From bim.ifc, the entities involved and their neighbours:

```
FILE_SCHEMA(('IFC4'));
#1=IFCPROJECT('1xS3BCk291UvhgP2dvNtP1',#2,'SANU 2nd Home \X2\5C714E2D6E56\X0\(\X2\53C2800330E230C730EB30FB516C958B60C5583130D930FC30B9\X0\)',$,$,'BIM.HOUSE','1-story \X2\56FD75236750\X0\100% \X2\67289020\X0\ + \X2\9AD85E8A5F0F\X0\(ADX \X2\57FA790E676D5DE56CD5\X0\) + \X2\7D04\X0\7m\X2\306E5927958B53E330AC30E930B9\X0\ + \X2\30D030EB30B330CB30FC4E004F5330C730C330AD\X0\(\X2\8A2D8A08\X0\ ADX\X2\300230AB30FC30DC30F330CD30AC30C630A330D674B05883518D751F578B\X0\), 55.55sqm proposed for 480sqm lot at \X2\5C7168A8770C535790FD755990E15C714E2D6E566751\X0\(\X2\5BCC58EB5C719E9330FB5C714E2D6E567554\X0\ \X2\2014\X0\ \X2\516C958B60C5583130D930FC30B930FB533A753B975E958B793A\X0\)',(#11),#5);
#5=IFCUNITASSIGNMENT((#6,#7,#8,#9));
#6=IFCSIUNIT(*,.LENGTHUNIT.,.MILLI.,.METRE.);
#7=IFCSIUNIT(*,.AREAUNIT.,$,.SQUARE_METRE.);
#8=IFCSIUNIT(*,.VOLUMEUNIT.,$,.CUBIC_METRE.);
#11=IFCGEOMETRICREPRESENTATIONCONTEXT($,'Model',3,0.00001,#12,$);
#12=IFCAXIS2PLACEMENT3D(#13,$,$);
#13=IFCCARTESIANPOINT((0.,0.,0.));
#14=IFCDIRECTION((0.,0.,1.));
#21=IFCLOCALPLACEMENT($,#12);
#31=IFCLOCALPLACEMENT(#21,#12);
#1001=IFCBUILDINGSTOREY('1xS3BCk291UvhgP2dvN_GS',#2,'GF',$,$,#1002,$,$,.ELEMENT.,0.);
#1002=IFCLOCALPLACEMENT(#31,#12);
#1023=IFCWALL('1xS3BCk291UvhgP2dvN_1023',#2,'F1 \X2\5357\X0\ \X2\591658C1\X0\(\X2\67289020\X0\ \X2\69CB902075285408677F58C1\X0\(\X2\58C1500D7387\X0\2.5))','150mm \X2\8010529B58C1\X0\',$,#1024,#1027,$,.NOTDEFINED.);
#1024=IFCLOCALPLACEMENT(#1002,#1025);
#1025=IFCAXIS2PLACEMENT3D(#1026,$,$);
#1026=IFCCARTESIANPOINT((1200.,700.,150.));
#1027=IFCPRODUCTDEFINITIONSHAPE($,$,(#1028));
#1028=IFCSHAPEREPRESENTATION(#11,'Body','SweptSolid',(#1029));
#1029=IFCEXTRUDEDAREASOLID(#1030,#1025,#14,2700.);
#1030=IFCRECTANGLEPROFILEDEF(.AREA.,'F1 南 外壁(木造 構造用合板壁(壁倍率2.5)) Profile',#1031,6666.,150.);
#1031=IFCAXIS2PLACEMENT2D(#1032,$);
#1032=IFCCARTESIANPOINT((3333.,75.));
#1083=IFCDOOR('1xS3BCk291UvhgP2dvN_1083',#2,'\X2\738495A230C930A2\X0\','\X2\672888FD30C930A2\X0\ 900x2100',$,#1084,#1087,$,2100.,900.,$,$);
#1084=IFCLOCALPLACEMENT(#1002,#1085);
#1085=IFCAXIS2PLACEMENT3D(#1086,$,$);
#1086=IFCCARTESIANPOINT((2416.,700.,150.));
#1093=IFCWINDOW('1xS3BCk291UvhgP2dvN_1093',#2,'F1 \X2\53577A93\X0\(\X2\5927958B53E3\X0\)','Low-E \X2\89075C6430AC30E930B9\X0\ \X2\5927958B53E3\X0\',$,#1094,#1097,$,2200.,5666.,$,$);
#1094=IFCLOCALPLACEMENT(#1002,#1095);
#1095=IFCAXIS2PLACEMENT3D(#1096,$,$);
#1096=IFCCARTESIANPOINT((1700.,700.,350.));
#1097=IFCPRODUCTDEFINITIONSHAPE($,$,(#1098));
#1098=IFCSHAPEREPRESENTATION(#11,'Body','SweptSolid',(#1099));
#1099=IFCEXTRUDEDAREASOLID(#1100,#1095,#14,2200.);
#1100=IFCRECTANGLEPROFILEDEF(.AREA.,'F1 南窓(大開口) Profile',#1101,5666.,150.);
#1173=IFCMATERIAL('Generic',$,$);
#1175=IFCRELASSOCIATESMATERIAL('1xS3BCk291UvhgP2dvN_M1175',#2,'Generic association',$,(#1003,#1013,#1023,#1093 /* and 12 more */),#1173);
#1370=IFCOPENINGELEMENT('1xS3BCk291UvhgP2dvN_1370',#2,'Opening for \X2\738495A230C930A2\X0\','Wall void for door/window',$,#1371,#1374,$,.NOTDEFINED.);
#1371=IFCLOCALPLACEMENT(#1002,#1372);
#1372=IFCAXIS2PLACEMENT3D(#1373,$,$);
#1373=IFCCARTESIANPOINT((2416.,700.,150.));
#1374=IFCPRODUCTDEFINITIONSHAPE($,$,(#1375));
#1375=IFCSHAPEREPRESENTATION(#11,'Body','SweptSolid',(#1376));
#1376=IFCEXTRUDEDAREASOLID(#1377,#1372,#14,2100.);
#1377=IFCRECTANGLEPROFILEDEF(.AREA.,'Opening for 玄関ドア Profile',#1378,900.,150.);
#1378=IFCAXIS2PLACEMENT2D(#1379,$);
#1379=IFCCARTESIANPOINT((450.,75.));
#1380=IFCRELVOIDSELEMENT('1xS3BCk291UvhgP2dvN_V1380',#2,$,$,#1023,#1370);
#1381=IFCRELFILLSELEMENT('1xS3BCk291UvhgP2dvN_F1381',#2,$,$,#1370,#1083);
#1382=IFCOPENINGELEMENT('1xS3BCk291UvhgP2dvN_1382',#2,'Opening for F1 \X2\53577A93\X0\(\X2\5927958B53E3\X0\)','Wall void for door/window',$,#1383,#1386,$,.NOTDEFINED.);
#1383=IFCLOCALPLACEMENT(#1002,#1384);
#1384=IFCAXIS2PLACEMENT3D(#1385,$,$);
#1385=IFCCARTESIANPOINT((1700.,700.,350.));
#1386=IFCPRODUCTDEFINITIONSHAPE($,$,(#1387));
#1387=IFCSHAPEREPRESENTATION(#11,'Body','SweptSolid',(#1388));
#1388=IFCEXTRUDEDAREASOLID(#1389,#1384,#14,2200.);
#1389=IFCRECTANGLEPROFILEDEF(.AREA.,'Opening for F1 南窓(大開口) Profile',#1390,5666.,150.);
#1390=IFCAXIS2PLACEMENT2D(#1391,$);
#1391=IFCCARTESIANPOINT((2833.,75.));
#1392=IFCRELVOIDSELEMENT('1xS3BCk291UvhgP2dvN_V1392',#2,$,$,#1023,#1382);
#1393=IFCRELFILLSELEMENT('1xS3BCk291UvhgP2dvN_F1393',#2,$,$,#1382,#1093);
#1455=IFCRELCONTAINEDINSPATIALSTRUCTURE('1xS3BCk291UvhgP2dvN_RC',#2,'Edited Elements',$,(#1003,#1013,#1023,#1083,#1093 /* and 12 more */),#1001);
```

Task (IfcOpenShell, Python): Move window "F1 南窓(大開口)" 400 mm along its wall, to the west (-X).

```python
import ifcopenshell
import ifcopenshell.api.geometry
import ifcopenshell.util.placement
import ifcopenshell.util.unit

model = ifcopenshell.open("bim.ifc")
unit_scale = ifcopenshell.util.unit.calculate_unit_scale(model)

window = model.by_guid("1xS3BCk291UvhgP2dvN_1093")
opening = window.FillsVoids[0].RelatingOpeningElement
wall = opening.VoidsElements[0].RelatingBuildingElement

wall_matrix = ifcopenshell.util.placement.get_local_placement(wall.ObjectPlacement)
shift = wall_matrix[:3, 0] * -0.4 / unit_scale
before = ifcopenshell.util.placement.get_local_placement(window.ObjectPlacement)[:3, 3].copy()

# The window is not placed relative to its opening, so move both.
for product in (opening, window):
    matrix = ifcopenshell.util.placement.get_local_placement(product.ObjectPlacement)
    matrix[:3, 3] += shift
    ifcopenshell.api.geometry.edit_object_placement(model, product=product, matrix=matrix, is_si=False)

after = ifcopenshell.util.placement.get_local_placement(window.ObjectPlacement)[:3, 3]
print("window moved by", (after - before).round(3) + 0.0)

model.write("bim_rev.ifc")
```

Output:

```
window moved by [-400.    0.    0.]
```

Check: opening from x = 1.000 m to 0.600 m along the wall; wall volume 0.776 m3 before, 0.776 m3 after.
